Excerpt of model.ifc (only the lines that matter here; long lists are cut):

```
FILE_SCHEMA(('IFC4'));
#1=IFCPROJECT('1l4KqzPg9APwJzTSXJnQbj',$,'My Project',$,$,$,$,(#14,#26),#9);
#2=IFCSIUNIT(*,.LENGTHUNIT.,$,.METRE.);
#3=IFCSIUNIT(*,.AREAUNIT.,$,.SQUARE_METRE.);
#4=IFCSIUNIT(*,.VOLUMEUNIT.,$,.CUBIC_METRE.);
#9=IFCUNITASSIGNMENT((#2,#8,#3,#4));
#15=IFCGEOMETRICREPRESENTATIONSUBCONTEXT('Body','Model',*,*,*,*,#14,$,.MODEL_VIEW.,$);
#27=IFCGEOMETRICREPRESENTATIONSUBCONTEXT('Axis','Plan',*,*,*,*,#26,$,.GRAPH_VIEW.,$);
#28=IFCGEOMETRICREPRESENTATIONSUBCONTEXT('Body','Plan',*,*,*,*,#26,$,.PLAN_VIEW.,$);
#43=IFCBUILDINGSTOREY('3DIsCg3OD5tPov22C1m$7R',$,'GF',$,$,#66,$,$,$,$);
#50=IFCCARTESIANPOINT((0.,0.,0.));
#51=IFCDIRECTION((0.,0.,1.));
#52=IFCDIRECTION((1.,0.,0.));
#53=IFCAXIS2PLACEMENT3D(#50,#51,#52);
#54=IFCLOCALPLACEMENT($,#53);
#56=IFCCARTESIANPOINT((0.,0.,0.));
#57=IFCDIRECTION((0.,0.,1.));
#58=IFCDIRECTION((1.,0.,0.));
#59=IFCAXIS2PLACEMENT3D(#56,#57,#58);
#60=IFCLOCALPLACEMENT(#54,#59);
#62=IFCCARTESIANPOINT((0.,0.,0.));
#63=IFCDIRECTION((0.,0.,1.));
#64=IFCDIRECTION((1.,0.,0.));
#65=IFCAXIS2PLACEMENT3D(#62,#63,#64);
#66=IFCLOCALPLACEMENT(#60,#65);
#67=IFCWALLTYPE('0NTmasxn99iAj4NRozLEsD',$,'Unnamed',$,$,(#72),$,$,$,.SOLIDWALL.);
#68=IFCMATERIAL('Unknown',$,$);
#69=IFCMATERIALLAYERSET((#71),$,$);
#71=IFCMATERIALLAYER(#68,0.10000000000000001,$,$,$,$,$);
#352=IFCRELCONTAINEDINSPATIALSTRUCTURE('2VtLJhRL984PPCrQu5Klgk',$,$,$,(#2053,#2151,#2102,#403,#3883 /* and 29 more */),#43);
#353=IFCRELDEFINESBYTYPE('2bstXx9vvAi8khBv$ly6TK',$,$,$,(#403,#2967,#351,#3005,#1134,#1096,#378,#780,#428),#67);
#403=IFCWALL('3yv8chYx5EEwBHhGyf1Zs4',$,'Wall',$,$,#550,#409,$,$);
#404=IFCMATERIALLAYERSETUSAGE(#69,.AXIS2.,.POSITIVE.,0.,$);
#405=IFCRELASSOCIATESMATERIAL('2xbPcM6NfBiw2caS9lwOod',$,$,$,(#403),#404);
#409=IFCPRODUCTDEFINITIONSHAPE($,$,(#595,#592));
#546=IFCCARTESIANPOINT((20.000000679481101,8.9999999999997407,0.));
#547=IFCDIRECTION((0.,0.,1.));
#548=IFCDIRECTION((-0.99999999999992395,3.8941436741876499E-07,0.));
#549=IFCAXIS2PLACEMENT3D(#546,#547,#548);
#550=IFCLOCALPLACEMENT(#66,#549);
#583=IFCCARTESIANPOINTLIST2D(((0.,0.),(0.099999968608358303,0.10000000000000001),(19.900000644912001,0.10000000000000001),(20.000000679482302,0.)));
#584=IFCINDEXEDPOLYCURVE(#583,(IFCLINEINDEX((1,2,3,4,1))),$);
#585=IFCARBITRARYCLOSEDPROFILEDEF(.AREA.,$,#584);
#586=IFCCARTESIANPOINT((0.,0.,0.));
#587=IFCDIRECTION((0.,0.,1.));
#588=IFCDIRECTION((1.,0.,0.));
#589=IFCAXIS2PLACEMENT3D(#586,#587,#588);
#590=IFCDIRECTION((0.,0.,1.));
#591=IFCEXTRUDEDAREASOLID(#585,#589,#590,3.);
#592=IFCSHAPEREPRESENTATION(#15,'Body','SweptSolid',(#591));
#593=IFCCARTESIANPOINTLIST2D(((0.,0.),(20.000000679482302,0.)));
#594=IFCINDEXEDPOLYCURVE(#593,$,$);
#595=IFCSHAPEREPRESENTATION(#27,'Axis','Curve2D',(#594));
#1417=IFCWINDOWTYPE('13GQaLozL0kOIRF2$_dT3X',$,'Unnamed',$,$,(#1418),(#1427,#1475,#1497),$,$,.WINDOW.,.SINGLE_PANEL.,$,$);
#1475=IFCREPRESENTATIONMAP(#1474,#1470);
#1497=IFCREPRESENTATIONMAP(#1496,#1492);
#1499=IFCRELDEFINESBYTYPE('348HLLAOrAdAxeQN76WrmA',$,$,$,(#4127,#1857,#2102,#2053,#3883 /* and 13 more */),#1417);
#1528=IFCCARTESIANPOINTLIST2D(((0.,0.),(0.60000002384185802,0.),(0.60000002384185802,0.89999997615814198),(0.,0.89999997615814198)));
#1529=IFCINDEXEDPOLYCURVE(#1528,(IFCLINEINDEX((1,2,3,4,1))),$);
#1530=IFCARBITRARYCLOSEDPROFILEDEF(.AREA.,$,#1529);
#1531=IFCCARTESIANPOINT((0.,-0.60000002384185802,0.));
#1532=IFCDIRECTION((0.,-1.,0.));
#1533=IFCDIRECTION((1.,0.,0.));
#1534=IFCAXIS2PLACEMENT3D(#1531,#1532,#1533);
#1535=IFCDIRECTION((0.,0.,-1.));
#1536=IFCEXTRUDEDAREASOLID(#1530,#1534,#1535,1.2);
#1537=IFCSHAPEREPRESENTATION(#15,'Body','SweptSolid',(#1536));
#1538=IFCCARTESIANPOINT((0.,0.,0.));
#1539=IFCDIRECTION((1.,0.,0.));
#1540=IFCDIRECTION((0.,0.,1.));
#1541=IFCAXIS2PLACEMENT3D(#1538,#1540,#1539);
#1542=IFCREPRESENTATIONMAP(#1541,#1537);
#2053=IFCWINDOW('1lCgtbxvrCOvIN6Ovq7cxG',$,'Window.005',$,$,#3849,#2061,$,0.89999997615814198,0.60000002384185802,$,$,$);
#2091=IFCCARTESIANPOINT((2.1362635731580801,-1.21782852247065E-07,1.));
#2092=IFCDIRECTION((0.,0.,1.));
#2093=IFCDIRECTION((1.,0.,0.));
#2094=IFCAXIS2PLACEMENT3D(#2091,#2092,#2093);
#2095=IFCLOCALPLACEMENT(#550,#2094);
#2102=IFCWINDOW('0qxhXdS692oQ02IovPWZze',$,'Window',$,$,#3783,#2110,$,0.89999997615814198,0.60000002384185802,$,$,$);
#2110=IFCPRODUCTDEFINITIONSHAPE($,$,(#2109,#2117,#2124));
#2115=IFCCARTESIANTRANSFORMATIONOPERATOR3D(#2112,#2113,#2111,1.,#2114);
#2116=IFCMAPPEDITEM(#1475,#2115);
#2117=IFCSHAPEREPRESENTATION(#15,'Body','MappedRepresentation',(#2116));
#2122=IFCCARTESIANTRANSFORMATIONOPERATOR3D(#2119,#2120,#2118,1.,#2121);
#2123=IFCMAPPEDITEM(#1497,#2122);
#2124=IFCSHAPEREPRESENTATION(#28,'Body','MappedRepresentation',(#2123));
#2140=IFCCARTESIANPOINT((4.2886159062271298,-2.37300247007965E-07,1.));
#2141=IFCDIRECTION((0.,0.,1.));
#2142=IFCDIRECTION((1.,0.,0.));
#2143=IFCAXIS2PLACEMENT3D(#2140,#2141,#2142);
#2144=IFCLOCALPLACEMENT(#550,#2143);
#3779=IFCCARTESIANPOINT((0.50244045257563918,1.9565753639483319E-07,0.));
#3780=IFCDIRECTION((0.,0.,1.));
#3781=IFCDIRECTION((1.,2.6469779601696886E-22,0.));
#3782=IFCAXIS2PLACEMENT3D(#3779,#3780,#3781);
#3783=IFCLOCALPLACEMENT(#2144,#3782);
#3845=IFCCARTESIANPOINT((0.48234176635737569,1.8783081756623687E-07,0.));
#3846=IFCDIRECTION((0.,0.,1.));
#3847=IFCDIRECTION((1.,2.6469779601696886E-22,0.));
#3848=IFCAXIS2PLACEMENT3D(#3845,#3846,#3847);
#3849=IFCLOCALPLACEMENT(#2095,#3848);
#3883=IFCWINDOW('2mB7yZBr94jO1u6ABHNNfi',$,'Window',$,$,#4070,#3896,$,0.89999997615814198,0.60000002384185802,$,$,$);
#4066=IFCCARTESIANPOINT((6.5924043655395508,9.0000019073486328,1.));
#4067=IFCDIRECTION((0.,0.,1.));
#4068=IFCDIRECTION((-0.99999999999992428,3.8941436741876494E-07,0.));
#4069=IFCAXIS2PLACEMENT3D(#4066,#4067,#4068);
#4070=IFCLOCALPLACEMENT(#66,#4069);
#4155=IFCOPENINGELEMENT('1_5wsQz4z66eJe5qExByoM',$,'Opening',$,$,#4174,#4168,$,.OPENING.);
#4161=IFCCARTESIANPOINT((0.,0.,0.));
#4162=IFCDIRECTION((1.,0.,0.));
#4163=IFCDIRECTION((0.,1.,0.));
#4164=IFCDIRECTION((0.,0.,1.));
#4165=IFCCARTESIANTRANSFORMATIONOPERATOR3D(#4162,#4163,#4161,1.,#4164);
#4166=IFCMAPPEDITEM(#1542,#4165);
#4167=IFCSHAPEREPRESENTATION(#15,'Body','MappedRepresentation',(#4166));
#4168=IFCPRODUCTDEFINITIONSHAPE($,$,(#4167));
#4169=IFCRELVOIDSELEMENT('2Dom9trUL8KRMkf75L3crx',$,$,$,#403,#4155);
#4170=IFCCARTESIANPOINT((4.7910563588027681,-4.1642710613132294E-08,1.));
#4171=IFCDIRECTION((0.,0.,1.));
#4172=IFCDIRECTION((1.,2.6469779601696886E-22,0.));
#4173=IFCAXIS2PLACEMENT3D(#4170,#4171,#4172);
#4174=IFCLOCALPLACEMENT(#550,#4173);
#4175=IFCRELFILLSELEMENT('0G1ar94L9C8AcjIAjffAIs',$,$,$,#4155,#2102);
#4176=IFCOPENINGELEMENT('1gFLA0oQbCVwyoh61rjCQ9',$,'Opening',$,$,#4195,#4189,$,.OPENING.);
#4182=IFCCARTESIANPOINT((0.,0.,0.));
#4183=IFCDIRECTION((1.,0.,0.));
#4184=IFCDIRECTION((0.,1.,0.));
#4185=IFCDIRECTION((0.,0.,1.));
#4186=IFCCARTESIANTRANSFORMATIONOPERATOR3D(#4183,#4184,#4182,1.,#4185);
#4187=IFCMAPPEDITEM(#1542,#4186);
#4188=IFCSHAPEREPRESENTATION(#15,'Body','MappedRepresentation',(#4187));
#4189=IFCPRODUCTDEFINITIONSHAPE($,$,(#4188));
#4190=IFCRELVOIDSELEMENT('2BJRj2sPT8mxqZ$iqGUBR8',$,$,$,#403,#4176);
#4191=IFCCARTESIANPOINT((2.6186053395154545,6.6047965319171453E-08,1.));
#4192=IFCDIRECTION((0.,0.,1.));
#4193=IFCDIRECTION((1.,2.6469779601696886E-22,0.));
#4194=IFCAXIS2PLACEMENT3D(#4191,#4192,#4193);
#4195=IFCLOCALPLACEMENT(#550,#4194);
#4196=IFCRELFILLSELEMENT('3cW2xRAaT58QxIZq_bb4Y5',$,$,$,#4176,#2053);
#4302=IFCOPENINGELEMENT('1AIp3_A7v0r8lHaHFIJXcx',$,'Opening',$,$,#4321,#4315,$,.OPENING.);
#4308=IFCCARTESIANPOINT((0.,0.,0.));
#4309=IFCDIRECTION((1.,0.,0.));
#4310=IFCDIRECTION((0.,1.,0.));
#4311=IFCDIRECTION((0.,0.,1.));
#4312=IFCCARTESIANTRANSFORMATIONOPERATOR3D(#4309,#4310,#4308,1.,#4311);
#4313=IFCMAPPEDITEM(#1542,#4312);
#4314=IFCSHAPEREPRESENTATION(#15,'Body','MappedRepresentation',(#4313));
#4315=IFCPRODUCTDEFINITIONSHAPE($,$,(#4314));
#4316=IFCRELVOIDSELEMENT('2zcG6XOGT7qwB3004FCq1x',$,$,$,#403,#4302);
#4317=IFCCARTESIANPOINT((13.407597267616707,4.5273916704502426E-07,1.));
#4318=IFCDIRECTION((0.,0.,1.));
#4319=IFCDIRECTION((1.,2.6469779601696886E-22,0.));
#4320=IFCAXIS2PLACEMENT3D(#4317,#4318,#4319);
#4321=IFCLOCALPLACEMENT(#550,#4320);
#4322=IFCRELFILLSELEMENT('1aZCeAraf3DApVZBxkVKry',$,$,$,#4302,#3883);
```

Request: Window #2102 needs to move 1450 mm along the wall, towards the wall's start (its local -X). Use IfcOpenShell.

```python
import ifcopenshell
import ifcopenshell.api.geometry
import ifcopenshell.util.placement

model = ifcopenshell.open("model.ifc")

window = model.by_guid("0qxhXdS692oQ02IovPWZze")
opening = window.FillsVoids[0].RelatingOpeningElement
wall = opening.VoidsElements[0].RelatingBuildingElement

wall_matrix = ifcopenshell.util.placement.get_local_placement(wall.ObjectPlacement)
shift = wall_matrix[:3, 0] * -1.45
before = ifcopenshell.util.placement.get_local_placement(window.ObjectPlacement)[:3, 3].copy()

# The window is not placed relative to its opening, so move both.
for product in (opening, window):
    matrix = ifcopenshell.util.placement.get_local_placement(product.ObjectPlacement)
    matrix[:3, 3] += shift
    ifcopenshell.api.geometry.edit_object_placement(model, product=product, matrix=matrix, is_si=False)

after = ifcopenshell.util.placement.get_local_placement(window.ObjectPlacement)[:3, 3]
print("window moved by", (after - before).round(3) + 0.0)

model.write("model_rev.ifc")
```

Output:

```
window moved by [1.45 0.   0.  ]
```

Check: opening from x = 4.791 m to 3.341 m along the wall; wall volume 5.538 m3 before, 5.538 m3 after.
